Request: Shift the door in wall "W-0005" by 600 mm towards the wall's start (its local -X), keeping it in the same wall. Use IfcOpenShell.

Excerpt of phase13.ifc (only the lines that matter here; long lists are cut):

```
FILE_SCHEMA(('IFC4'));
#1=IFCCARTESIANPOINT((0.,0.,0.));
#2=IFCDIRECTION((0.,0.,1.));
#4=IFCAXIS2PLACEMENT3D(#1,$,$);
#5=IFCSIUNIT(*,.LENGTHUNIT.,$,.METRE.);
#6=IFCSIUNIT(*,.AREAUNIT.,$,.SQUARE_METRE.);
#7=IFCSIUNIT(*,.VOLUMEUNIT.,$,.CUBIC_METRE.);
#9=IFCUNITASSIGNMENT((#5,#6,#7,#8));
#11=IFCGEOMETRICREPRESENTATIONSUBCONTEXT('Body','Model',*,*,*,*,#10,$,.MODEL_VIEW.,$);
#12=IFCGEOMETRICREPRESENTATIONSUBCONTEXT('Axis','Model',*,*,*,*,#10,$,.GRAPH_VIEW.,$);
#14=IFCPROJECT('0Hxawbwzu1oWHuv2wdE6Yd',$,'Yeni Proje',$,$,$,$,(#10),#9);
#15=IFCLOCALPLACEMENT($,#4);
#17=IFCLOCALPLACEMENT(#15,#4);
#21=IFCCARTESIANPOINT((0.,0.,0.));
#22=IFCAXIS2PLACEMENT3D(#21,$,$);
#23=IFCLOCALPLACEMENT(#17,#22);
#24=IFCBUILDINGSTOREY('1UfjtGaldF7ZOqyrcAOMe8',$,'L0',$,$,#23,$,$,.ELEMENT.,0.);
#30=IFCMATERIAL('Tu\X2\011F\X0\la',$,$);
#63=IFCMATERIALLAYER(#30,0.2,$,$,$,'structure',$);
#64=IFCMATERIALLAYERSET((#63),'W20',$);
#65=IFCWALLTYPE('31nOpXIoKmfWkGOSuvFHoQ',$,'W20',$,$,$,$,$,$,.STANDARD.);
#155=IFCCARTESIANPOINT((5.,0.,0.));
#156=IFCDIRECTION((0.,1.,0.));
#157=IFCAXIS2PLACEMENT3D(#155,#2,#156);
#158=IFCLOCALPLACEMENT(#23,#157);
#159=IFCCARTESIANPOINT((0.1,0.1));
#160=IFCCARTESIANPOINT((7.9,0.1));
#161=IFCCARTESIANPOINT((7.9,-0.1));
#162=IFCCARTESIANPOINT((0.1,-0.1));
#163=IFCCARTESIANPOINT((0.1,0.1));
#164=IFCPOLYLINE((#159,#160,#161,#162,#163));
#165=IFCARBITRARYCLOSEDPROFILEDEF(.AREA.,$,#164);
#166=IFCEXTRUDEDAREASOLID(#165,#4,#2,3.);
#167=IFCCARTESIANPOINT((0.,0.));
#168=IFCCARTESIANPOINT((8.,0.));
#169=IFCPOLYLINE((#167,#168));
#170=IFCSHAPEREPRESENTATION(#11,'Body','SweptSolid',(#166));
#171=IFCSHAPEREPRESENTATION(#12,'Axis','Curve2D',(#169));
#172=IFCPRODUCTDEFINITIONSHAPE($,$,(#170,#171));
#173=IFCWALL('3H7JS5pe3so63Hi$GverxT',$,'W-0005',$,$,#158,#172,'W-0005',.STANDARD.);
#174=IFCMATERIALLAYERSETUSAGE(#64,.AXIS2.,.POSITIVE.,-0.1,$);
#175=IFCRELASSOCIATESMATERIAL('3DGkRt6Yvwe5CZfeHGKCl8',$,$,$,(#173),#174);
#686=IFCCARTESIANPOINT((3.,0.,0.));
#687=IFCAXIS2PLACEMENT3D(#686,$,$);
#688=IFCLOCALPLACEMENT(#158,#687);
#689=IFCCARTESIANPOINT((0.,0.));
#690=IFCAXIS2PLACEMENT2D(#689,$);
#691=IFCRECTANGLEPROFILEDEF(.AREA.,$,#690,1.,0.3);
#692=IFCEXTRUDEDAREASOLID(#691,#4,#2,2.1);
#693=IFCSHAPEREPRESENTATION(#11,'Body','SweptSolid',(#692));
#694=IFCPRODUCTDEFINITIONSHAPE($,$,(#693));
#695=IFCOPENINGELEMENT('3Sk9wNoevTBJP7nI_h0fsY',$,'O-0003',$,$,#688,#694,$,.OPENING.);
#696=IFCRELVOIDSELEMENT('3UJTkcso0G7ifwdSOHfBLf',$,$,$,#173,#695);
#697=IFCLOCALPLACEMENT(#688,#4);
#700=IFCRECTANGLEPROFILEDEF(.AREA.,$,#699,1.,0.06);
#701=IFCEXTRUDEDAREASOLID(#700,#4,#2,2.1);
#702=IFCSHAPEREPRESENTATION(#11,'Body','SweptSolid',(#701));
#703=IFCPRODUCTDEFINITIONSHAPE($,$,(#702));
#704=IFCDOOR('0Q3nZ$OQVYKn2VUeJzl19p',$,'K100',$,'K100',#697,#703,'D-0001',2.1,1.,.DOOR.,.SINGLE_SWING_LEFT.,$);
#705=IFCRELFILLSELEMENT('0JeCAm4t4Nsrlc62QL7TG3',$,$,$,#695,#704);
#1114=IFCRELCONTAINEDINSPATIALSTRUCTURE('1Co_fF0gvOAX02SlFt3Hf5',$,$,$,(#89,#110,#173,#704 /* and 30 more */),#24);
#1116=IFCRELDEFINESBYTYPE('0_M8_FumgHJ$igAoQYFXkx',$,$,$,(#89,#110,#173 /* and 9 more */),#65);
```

```python
import ifcopenshell
import ifcopenshell.api.geometry
import ifcopenshell.util.placement
import ifcopenshell.util.unit

model = ifcopenshell.open("phase13.ifc")
unit_scale = ifcopenshell.util.unit.calculate_unit_scale(model)

door = model.by_guid("0Q3nZ$OQVYKn2VUeJzl19p")
opening = door.FillsVoids[0].RelatingOpeningElement
wall = opening.VoidsElements[0].RelatingBuildingElement

wall_matrix = ifcopenshell.util.placement.get_local_placement(wall.ObjectPlacement)
shift = wall_matrix[:3, 0] * -0.6 / unit_scale
before = ifcopenshell.util.placement.get_local_placement(door.ObjectPlacement)[:3, 3].copy()

# The door is placed relative to its opening, so it follows when the opening moves.
matrix = ifcopenshell.util.placement.get_local_placement(opening.ObjectPlacement)
matrix[:3, 3] += shift
ifcopenshell.api.geometry.edit_object_placement(
    model, product=opening, matrix=matrix, is_si=False, should_transform_children=True
)

after = ifcopenshell.util.placement.get_local_placement(door.ObjectPlacement)[:3, 3]
print("door moved by", (after - before).round(3) + 0.0)

model.write("phase13_v2.ifc")
```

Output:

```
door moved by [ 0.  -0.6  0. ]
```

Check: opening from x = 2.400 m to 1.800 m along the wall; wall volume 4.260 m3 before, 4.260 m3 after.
